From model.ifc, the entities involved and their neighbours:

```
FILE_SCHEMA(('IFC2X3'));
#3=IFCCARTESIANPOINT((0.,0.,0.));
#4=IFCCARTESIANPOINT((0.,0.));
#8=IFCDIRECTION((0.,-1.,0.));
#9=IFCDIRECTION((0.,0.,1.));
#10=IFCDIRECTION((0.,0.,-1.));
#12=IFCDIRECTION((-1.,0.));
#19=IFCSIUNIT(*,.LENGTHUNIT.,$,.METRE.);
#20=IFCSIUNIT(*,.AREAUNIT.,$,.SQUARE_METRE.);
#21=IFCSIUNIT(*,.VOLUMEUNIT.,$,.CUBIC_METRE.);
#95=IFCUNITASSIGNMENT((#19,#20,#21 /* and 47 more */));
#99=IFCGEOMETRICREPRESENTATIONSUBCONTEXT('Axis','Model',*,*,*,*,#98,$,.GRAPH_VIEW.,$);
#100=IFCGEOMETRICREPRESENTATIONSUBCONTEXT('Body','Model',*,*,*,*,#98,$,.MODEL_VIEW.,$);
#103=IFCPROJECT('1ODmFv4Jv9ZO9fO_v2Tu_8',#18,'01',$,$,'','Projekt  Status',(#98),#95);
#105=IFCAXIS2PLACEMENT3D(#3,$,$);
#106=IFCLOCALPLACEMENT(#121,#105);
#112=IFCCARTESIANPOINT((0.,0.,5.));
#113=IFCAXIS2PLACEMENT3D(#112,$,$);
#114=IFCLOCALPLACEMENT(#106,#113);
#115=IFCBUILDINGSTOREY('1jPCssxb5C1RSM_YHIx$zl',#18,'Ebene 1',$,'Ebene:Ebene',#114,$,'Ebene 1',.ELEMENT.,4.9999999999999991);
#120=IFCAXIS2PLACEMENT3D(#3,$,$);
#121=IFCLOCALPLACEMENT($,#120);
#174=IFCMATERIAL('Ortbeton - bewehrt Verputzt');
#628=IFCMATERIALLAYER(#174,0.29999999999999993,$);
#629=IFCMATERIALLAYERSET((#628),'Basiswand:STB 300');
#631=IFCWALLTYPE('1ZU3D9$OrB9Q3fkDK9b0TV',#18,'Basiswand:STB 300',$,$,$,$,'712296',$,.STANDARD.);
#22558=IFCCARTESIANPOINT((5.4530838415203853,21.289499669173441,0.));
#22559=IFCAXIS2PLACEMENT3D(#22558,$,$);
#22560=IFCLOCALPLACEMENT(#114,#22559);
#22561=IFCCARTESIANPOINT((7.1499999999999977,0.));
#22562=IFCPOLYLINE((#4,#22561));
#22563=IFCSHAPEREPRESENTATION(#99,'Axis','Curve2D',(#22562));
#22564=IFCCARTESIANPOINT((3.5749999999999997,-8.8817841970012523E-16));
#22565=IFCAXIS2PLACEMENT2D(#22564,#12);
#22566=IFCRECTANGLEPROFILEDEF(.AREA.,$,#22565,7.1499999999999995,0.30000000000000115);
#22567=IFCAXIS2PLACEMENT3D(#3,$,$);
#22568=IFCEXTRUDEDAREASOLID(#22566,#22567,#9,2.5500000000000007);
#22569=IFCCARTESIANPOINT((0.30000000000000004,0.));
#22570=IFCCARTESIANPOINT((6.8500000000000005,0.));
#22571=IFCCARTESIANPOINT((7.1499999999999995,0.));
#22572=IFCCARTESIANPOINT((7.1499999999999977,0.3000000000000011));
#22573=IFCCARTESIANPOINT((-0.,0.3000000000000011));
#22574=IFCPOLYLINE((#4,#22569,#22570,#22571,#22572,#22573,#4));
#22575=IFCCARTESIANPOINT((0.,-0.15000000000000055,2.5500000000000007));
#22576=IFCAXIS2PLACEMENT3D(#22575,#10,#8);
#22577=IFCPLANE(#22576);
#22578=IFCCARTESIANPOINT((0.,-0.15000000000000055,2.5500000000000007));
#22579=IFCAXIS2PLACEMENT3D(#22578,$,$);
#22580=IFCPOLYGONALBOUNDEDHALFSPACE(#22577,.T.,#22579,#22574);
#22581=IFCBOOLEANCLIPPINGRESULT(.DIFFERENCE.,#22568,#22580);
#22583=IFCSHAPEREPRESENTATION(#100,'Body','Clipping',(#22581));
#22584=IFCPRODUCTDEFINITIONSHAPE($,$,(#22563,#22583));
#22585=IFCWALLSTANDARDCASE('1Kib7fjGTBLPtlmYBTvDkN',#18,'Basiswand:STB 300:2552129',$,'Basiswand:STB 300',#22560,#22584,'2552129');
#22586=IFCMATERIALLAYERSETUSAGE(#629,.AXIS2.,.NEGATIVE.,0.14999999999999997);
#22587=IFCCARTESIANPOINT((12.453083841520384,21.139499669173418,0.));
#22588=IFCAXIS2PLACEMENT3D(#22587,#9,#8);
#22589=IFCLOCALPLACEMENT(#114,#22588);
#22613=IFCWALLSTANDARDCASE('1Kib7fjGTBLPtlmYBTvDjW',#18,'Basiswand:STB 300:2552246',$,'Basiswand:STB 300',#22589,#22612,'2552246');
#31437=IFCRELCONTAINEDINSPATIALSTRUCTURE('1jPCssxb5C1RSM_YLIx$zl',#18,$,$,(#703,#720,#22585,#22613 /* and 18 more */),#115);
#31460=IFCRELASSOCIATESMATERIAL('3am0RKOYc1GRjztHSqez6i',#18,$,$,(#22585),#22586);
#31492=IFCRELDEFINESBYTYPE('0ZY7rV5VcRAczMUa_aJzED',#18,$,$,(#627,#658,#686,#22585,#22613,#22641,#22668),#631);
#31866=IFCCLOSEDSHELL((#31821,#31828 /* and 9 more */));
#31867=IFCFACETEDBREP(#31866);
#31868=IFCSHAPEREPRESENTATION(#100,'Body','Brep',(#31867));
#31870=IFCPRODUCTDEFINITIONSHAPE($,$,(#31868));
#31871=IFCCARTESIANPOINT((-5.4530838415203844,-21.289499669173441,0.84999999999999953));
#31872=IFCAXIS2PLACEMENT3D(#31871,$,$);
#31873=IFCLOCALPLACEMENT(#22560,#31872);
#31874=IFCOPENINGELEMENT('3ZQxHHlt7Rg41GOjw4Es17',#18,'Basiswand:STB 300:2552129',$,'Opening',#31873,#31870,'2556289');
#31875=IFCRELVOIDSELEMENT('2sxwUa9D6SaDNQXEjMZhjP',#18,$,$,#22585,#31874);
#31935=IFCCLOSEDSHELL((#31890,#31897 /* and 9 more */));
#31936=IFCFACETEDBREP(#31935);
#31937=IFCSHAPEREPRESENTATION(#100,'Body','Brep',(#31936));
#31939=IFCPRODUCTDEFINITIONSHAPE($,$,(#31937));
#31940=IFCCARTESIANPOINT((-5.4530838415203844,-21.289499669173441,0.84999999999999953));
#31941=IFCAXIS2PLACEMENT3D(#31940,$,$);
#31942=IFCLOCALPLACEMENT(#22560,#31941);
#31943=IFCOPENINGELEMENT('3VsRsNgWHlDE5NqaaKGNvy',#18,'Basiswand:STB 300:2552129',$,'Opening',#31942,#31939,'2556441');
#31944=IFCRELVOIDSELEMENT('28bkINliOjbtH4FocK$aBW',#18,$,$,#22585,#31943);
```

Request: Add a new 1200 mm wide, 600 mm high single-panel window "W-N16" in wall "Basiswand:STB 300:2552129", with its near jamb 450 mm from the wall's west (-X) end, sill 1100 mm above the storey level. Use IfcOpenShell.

```python
import numpy as np
import ifcopenshell
import ifcopenshell.api.feature
import ifcopenshell.api.geometry
import ifcopenshell.api.root
import ifcopenshell.api.spatial
import ifcopenshell.api.type
import ifcopenshell.geom
import ifcopenshell.util.element
import ifcopenshell.util.placement
import ifcopenshell.util.representation
import ifcopenshell.util.shape
import ifcopenshell.util.unit

model = ifcopenshell.open("model.ifc")
unit_scale = ifcopenshell.util.unit.calculate_unit_scale(model)
settings = ifcopenshell.geom.settings()


def volume(element):
    """Net volume in cubic metres, openings subtracted."""
    shape = ifcopenshell.geom.create_shape(settings, element)
    return ifcopenshell.util.shape.get_volume(shape.geometry)


wall = model.by_id(22585)
storey = ifcopenshell.util.element.get_container(wall, ifc_class="IfcBuildingStorey")
context = ifcopenshell.util.representation.get_context(model, "Model", "Body", "MODEL_VIEW")
before = volume(wall)

width, height, from_end, sill = 1.2, 0.6, 0.45, 1.1  # metres

# The wall runs along its own X axis, and the end named is its -X end.
wall_shape = ifcopenshell.geom.create_shape(settings, wall)
x, y, z = ifcopenshell.util.shape.get_vertices(wall_shape.geometry).T
start = x.min() + from_end
face, thickness = float(y.min()), float(y.max() - y.min())
wall_matrix = ifcopenshell.util.placement.get_local_placement(wall.ObjectPlacement)
level = ifcopenshell.util.placement.get_local_placement(storey.ObjectPlacement)[2, 3]


def in_wall(x, y):
    """Placement at x, y metres in the wall's axes, at sill height."""
    matrix = wall_matrix.copy()
    matrix[:, 3] = wall_matrix @ np.array([x / unit_scale, y / unit_scale, 0.0, 1.0])
    matrix[2, 3] = level + sill / unit_scale
    return matrix


# Opening: a box that overshoots both wall faces by 50 mm.
opening = ifcopenshell.api.root.create_entity(model, ifc_class="IfcOpeningElement")
box = ifcopenshell.api.geometry.add_wall_representation(
    model, context=context, length=width, height=height, thickness=thickness + 0.1
)
ifcopenshell.api.geometry.assign_representation(model, product=opening, representation=box)
ifcopenshell.api.geometry.edit_object_placement(model, product=opening, matrix=in_wall(start, face - 0.05), is_si=False)
ifcopenshell.api.feature.add_feature(model, feature=opening, element=wall)

window = ifcopenshell.api.root.create_entity(model, ifc_class="IfcWindow", name="W-N16")
window.OverallWidth, window.OverallHeight = width / unit_scale, height / unit_scale
body = ifcopenshell.api.geometry.add_window_representation(
    model,
    context=context,
    overall_width=window.OverallWidth,
    overall_height=window.OverallHeight,
    partition_type="SINGLE_PANEL",
)
ifcopenshell.api.geometry.assign_representation(model, product=window, representation=body)
ifcopenshell.api.spatial.assign_container(model, products=[window], relating_structure=storey)
fills = ifcopenshell.api.feature.add_filling(model, opening=opening, element=window)
fills.OwnerHistory = window.OwnerHistory  # required in IFC2X3

# IFC2X3 keeps the operation on the window style.
style = ifcopenshell.api.root.create_entity(model, ifc_class="IfcWindowStyle", name="W-N16")
style.OperationType, style.ConstructionType = "SINGLE_PANEL", "NOTDEFINED"
style.ParameterTakesPrecedence = style.Sizeable = False
ifcopenshell.api.type.assign_type(model, related_objects=[window], relating_type=style)

# Centre the window in the wall's thickness.
ifcopenshell.api.geometry.edit_object_placement(model, product=window, matrix=in_wall(start, face), is_si=False)
window_shape = ifcopenshell.geom.create_shape(settings, window)
depth = ifcopenshell.util.shape.get_vertices(window_shape.geometry)[:, 1]
offset = face + thickness / 2 - (depth.min() + depth.max()) / 2
ifcopenshell.api.geometry.edit_object_placement(model, product=window, matrix=in_wall(start, offset), is_si=False)

after = volume(wall)

print(f"wall volume {before:.3f} -> {after:.3f} m3")

model.write("model_v2.ifc")
```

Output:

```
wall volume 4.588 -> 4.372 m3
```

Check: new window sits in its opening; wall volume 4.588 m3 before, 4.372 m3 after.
